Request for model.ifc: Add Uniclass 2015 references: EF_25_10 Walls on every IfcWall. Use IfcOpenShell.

First a look at what the model holds.

```python
import ifcopenshell

model = ifcopenshell.open("model.ifc")
print(model.schema)
print("classifications:", [c.Name for c in model.by_type("IfcClassification")])
for ifc_class in ("IfcDoor", "IfcRoof", "IfcStair", "IfcWall", "IfcWindow"):
    print(ifc_class, len(model.by_type(ifc_class)))
```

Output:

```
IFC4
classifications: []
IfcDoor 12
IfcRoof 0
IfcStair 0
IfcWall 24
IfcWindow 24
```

```python
import ifcopenshell
import ifcopenshell.api.classification

model = ifcopenshell.open("model.ifc")

system = ifcopenshell.api.classification.add_classification(model, classification="Uniclass 2015")

codes = {
    "IfcWall": ("EF_25_10", "Walls"),
}
for ifc_class, (code, name) in codes.items():
    products = model.by_type(ifc_class)
    ifcopenshell.api.classification.add_reference(
        model, products=products, classification=system, identification=code, name=name
    )
    print(code, len(products))

model.write("model_v2.ifc")
```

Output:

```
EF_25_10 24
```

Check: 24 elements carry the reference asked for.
